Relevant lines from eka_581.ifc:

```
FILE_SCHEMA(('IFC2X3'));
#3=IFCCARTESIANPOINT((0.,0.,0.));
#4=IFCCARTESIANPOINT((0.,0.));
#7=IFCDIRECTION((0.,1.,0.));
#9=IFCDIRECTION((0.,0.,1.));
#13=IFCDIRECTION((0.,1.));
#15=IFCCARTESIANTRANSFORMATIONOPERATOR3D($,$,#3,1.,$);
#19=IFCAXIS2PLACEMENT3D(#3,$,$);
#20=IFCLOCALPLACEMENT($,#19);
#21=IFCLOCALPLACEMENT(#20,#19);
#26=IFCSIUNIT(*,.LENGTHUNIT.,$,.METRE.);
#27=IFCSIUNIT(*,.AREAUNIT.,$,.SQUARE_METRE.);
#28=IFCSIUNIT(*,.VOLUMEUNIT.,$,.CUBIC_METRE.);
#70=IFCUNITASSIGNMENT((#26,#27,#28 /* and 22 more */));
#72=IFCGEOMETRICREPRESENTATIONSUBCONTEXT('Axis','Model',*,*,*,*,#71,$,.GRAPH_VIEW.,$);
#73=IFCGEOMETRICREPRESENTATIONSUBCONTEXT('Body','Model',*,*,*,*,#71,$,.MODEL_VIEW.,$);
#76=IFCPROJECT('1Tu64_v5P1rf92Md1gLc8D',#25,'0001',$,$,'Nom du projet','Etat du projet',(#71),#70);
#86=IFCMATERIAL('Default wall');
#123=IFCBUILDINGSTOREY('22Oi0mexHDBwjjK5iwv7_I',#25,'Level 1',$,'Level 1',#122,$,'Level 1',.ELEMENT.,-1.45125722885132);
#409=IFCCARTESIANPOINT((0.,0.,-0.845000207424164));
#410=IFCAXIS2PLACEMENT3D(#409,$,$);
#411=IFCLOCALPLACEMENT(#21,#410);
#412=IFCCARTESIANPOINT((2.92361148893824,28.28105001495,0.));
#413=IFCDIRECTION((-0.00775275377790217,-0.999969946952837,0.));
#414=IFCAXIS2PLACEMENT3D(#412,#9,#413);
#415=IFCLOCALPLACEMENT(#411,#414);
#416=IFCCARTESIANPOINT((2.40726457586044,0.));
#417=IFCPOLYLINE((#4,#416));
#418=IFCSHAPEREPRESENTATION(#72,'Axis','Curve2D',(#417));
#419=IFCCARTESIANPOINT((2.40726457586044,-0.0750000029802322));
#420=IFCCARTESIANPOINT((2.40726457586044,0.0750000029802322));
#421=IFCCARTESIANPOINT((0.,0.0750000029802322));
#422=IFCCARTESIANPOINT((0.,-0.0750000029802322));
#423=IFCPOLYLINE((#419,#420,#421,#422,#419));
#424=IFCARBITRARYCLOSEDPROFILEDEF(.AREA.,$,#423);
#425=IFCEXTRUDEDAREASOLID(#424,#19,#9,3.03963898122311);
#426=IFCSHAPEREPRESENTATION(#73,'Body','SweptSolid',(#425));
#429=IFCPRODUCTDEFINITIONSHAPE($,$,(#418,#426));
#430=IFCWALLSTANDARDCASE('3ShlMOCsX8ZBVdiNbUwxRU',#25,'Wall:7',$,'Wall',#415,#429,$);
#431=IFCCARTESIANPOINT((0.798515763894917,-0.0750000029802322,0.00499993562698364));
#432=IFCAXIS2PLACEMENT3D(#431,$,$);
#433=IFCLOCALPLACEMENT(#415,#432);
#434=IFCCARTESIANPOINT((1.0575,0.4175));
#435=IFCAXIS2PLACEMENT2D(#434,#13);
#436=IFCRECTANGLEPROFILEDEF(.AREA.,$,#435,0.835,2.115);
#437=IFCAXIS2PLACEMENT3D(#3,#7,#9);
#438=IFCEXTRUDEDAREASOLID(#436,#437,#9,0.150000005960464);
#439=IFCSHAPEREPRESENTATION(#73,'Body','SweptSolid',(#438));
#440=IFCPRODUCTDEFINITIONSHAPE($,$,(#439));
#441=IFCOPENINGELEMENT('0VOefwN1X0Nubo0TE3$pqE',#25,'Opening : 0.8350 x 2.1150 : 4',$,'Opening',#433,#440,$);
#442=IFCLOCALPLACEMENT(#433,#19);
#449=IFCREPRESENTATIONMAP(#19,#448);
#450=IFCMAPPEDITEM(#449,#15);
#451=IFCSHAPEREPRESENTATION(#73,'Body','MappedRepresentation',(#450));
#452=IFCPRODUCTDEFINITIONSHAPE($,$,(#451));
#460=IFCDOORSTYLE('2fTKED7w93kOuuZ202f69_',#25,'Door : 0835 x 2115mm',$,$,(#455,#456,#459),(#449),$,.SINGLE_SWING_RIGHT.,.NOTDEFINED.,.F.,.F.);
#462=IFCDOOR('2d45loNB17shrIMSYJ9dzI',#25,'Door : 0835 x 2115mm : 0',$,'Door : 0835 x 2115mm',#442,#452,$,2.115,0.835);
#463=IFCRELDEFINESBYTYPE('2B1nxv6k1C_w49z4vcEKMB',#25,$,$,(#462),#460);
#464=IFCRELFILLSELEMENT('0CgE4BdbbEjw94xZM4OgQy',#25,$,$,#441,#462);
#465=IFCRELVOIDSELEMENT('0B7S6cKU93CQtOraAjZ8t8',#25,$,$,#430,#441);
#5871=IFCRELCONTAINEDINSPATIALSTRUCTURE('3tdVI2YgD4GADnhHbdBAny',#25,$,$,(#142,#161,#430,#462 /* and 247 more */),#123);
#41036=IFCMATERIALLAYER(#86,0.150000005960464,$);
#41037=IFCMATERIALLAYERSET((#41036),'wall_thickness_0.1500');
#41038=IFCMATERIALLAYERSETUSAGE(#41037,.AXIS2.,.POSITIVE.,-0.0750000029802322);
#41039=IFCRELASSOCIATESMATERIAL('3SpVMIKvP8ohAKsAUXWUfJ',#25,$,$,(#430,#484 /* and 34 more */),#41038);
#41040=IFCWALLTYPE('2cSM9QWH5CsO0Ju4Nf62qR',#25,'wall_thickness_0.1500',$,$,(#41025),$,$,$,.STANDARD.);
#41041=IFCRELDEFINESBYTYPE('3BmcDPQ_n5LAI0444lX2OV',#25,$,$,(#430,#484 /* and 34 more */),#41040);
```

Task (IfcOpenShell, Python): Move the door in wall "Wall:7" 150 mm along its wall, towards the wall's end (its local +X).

```python
import ifcopenshell
import ifcopenshell.api.geometry
import ifcopenshell.util.placement

model = ifcopenshell.open("eka_581.ifc")

door = model.by_guid("2d45loNB17shrIMSYJ9dzI")
opening = door.FillsVoids[0].RelatingOpeningElement
wall = opening.VoidsElements[0].RelatingBuildingElement

wall_matrix = ifcopenshell.util.placement.get_local_placement(wall.ObjectPlacement)
shift = wall_matrix[:3, 0] * 0.15
before = ifcopenshell.util.placement.get_local_placement(door.ObjectPlacement)[:3, 3].copy()

# The door is placed relative to its opening, so it follows when the opening moves.
matrix = ifcopenshell.util.placement.get_local_placement(opening.ObjectPlacement)
matrix[:3, 3] += shift
ifcopenshell.api.geometry.edit_object_placement(
    model, product=opening, matrix=matrix, is_si=False, should_transform_children=True
)

after = ifcopenshell.util.placement.get_local_placement(door.ObjectPlacement)[:3, 3]
print("door moved by", (after - before).round(3) + 0.0)

model.write("eka_581_edited.ifc")
```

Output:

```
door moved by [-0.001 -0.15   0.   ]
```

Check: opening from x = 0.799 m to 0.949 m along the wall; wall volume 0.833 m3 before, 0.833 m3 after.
